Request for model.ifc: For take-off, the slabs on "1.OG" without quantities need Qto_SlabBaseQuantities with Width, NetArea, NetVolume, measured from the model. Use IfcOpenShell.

First a look at what the model holds.

```python
import ifcopenshell
import ifcopenshell.util.element
import ifcopenshell.util.unit

model = ifcopenshell.open("model.ifc")
print(model.schema)
for unit_type in ("LENGTHUNIT", "AREAUNIT", "VOLUMEUNIT"):
    print(unit_type, ifcopenshell.util.unit.calculate_unit_scale(model, unit_type))
storey = next(s for s in model.by_type("IfcBuildingStorey") if s.Name == "1.OG")
slabs = [e for e in ifcopenshell.util.element.get_decomposition(storey) if e.is_a("IfcSlab")]
for e in sorted(slabs, key=lambda e: e.id()):
    print(e.id(), e.is_a(), e.Name, list(ifcopenshell.util.element.get_psets(e, qtos_only=True)), sep=" | ")
```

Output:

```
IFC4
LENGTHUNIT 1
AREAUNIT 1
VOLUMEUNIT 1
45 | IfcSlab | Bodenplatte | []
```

```python
import ifcopenshell
import ifcopenshell.api.pset
import ifcopenshell.geom
import ifcopenshell.util.element
import ifcopenshell.util.shape
import ifcopenshell.util.unit

model = ifcopenshell.open("model.ifc")
unit_scale = ifcopenshell.util.unit.calculate_unit_scale(model)
area_scale = ifcopenshell.util.unit.calculate_unit_scale(model, "AREAUNIT")
volume_scale = ifcopenshell.util.unit.calculate_unit_scale(model, "VOLUMEUNIT")
settings = ifcopenshell.geom.settings()

storey = next(s for s in model.by_type("IfcBuildingStorey") if s.Name == "1.OG")
slabs = [e for e in ifcopenshell.util.element.get_decomposition(storey) if e.is_a("IfcSlab")]

for e in sorted(slabs, key=lambda e: e.id()):
    if ifcopenshell.util.element.get_psets(e, qtos_only=True, should_inherit=False):
        continue
    # Geometry comes back in metres, in the element's own axes.
    shape = ifcopenshell.geom.create_shape(settings, e)
    values = {
        "Width": ifcopenshell.util.shape.get_z(shape.geometry) / unit_scale,
        "NetArea": ifcopenshell.util.shape.get_footprint_area(shape.geometry) / area_scale,
        "NetVolume": ifcopenshell.util.shape.get_volume(shape.geometry) / volume_scale,
    }
    qto = ifcopenshell.api.pset.add_qto(model, product=e, name="Qto_SlabBaseQuantities")
    ifcopenshell.api.pset.edit_qto(model, qto=qto, properties=values)
    print(e.id(), {k: round(v, 3) for k, v in values.items()})

model.write("model_updated.ifc")
```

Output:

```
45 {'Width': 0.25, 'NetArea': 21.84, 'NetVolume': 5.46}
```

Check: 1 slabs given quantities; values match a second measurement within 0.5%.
